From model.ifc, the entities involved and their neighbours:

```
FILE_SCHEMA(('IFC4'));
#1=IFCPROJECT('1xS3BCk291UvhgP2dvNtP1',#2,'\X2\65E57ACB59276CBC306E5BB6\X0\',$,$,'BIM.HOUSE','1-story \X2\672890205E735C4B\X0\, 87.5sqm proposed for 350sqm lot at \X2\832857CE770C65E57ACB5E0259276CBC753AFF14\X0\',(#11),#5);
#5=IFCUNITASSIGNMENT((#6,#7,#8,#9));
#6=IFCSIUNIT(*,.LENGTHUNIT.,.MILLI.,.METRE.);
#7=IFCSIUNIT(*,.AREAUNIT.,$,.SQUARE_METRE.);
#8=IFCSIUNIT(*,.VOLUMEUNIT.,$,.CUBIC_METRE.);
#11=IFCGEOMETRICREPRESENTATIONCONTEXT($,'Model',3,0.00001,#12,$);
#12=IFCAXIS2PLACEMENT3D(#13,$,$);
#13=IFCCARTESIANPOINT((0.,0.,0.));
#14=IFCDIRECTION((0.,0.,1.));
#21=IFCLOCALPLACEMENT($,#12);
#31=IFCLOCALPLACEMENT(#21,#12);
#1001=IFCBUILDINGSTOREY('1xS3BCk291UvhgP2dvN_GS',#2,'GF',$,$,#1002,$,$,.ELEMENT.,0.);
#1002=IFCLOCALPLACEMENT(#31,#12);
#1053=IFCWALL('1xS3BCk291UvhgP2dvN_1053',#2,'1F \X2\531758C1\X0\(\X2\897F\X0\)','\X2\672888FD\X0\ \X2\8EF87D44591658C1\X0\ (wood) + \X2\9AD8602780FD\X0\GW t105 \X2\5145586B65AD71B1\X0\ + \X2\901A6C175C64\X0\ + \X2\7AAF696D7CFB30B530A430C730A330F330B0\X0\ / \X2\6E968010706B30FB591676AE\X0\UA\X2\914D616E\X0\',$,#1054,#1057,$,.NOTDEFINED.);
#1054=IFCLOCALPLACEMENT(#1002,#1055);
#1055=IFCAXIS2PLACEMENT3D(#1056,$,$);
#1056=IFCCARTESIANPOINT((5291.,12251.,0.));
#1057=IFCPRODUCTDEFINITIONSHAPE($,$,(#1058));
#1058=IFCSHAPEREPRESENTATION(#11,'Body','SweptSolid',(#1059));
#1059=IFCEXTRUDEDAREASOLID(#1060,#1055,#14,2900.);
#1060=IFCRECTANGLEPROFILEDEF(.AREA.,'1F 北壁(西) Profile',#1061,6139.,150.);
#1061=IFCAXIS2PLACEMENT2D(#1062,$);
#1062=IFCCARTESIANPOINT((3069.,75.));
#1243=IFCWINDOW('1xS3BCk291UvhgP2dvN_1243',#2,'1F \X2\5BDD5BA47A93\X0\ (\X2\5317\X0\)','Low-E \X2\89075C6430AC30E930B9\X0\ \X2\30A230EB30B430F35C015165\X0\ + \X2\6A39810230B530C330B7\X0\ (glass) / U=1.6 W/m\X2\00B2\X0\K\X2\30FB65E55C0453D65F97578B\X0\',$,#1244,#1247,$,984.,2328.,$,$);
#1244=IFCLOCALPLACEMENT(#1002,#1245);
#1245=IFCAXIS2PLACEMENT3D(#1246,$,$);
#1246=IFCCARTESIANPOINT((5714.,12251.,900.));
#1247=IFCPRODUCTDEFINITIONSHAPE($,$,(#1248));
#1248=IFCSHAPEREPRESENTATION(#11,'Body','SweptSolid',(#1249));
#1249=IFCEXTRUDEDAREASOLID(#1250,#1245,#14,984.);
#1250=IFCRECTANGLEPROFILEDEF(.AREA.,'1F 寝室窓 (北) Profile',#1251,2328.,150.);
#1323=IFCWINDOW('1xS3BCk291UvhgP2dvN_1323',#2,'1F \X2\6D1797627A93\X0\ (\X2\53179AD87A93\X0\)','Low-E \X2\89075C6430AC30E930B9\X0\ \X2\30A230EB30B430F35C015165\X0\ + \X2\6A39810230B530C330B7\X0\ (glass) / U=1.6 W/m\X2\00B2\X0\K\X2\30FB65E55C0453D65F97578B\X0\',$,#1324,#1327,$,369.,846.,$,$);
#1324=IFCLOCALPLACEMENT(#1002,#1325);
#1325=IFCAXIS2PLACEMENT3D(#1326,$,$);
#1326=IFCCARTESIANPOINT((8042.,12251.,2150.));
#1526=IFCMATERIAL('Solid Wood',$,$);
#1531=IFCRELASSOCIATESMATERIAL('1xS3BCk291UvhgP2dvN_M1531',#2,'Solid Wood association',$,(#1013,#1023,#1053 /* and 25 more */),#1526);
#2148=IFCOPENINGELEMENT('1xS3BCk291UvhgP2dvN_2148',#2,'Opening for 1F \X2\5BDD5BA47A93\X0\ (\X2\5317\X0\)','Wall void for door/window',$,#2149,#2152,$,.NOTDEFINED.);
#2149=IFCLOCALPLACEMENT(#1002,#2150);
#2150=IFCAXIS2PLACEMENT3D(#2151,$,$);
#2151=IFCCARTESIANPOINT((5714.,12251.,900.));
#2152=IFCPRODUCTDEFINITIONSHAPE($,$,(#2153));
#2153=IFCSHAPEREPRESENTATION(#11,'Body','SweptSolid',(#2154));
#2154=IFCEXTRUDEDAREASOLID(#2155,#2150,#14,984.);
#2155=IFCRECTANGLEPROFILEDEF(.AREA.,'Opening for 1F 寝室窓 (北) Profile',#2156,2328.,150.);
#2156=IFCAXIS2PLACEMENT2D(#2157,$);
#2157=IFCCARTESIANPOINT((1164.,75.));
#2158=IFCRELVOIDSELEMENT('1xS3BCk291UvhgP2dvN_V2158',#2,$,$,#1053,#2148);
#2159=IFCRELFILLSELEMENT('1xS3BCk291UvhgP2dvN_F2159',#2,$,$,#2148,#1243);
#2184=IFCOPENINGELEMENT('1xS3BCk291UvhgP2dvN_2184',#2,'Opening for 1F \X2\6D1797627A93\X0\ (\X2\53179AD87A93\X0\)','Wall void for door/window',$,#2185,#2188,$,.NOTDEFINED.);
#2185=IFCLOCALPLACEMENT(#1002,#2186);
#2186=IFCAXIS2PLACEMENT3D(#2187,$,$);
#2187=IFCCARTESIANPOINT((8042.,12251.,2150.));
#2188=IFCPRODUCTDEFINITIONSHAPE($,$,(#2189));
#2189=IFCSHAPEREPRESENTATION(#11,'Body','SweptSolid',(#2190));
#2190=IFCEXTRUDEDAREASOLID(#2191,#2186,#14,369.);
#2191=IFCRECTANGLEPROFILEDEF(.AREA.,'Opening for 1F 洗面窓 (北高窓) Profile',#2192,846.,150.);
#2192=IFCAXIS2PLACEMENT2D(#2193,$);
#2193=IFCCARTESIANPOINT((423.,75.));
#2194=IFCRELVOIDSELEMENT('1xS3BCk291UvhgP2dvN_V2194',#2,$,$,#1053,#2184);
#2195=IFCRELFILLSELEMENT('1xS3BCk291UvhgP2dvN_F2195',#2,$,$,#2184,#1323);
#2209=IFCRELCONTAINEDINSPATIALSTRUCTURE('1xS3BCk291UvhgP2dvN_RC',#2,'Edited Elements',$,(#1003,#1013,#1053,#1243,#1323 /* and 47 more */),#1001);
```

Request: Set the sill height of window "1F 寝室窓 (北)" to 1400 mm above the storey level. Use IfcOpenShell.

```python
import numpy as np
import ifcopenshell
import ifcopenshell.api.geometry
import ifcopenshell.geom
import ifcopenshell.util.element
import ifcopenshell.util.placement
import ifcopenshell.util.shape
import ifcopenshell.util.unit

model = ifcopenshell.open("model.ifc")
unit_scale = ifcopenshell.util.unit.calculate_unit_scale(model)

window = model.by_guid("1xS3BCk291UvhgP2dvN_1243")
opening = window.FillsVoids[0].RelatingOpeningElement
storey = ifcopenshell.util.element.get_container(window, ifc_class="IfcBuildingStorey")
level = ifcopenshell.util.placement.get_local_placement(storey.ObjectPlacement)[2, 3]

# The opening's origin need not be at the sill, so measure its lowest point.
shape = ifcopenshell.geom.create_shape(ifcopenshell.geom.settings(), opening)
bottom = ifcopenshell.util.shape.get_shape_bottom_elevation(shape, shape.geometry) / unit_scale
dz = level + 1400.0 - bottom

shift = np.array([0.0, 0.0, dz])
# The window is not placed relative to its opening, so move both.
for product in (opening, window):
    matrix = ifcopenshell.util.placement.get_local_placement(product.ObjectPlacement)
    matrix[:3, 3] += shift
    ifcopenshell.api.geometry.edit_object_placement(model, product=product, matrix=matrix, is_si=False)

print(f"moved by {dz * unit_scale:+.3f} m")

model.write("model_rev.ifc")
```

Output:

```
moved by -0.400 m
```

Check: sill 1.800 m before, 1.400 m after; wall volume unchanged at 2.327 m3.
